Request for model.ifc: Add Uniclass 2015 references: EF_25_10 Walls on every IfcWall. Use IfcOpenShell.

First a look at what the model holds.

```python
import ifcopenshell

model = ifcopenshell.open("model.ifc")
print(model.schema)
print("classifications:", [c.Name for c in model.by_type("IfcClassification")])
for ifc_class in ("IfcDoor", "IfcRoof", "IfcStair", "IfcWall", "IfcWindow"):
    print(ifc_class, len(model.by_type(ifc_class)))
```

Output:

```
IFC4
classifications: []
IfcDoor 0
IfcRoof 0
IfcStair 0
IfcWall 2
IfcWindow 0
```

```python
import ifcopenshell
import ifcopenshell.api.classification

model = ifcopenshell.open("model.ifc")

system = ifcopenshell.api.classification.add_classification(model, classification="Uniclass 2015")

codes = {
    "IfcWall": ("EF_25_10", "Walls"),
}
for ifc_class, (code, name) in codes.items():
    products = model.by_type(ifc_class)
    ifcopenshell.api.classification.add_reference(
        model, products=products, classification=system, identification=code, name=name
    )
    print(code, len(products))

model.write("model_updated.ifc")
```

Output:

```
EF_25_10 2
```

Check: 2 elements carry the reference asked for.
